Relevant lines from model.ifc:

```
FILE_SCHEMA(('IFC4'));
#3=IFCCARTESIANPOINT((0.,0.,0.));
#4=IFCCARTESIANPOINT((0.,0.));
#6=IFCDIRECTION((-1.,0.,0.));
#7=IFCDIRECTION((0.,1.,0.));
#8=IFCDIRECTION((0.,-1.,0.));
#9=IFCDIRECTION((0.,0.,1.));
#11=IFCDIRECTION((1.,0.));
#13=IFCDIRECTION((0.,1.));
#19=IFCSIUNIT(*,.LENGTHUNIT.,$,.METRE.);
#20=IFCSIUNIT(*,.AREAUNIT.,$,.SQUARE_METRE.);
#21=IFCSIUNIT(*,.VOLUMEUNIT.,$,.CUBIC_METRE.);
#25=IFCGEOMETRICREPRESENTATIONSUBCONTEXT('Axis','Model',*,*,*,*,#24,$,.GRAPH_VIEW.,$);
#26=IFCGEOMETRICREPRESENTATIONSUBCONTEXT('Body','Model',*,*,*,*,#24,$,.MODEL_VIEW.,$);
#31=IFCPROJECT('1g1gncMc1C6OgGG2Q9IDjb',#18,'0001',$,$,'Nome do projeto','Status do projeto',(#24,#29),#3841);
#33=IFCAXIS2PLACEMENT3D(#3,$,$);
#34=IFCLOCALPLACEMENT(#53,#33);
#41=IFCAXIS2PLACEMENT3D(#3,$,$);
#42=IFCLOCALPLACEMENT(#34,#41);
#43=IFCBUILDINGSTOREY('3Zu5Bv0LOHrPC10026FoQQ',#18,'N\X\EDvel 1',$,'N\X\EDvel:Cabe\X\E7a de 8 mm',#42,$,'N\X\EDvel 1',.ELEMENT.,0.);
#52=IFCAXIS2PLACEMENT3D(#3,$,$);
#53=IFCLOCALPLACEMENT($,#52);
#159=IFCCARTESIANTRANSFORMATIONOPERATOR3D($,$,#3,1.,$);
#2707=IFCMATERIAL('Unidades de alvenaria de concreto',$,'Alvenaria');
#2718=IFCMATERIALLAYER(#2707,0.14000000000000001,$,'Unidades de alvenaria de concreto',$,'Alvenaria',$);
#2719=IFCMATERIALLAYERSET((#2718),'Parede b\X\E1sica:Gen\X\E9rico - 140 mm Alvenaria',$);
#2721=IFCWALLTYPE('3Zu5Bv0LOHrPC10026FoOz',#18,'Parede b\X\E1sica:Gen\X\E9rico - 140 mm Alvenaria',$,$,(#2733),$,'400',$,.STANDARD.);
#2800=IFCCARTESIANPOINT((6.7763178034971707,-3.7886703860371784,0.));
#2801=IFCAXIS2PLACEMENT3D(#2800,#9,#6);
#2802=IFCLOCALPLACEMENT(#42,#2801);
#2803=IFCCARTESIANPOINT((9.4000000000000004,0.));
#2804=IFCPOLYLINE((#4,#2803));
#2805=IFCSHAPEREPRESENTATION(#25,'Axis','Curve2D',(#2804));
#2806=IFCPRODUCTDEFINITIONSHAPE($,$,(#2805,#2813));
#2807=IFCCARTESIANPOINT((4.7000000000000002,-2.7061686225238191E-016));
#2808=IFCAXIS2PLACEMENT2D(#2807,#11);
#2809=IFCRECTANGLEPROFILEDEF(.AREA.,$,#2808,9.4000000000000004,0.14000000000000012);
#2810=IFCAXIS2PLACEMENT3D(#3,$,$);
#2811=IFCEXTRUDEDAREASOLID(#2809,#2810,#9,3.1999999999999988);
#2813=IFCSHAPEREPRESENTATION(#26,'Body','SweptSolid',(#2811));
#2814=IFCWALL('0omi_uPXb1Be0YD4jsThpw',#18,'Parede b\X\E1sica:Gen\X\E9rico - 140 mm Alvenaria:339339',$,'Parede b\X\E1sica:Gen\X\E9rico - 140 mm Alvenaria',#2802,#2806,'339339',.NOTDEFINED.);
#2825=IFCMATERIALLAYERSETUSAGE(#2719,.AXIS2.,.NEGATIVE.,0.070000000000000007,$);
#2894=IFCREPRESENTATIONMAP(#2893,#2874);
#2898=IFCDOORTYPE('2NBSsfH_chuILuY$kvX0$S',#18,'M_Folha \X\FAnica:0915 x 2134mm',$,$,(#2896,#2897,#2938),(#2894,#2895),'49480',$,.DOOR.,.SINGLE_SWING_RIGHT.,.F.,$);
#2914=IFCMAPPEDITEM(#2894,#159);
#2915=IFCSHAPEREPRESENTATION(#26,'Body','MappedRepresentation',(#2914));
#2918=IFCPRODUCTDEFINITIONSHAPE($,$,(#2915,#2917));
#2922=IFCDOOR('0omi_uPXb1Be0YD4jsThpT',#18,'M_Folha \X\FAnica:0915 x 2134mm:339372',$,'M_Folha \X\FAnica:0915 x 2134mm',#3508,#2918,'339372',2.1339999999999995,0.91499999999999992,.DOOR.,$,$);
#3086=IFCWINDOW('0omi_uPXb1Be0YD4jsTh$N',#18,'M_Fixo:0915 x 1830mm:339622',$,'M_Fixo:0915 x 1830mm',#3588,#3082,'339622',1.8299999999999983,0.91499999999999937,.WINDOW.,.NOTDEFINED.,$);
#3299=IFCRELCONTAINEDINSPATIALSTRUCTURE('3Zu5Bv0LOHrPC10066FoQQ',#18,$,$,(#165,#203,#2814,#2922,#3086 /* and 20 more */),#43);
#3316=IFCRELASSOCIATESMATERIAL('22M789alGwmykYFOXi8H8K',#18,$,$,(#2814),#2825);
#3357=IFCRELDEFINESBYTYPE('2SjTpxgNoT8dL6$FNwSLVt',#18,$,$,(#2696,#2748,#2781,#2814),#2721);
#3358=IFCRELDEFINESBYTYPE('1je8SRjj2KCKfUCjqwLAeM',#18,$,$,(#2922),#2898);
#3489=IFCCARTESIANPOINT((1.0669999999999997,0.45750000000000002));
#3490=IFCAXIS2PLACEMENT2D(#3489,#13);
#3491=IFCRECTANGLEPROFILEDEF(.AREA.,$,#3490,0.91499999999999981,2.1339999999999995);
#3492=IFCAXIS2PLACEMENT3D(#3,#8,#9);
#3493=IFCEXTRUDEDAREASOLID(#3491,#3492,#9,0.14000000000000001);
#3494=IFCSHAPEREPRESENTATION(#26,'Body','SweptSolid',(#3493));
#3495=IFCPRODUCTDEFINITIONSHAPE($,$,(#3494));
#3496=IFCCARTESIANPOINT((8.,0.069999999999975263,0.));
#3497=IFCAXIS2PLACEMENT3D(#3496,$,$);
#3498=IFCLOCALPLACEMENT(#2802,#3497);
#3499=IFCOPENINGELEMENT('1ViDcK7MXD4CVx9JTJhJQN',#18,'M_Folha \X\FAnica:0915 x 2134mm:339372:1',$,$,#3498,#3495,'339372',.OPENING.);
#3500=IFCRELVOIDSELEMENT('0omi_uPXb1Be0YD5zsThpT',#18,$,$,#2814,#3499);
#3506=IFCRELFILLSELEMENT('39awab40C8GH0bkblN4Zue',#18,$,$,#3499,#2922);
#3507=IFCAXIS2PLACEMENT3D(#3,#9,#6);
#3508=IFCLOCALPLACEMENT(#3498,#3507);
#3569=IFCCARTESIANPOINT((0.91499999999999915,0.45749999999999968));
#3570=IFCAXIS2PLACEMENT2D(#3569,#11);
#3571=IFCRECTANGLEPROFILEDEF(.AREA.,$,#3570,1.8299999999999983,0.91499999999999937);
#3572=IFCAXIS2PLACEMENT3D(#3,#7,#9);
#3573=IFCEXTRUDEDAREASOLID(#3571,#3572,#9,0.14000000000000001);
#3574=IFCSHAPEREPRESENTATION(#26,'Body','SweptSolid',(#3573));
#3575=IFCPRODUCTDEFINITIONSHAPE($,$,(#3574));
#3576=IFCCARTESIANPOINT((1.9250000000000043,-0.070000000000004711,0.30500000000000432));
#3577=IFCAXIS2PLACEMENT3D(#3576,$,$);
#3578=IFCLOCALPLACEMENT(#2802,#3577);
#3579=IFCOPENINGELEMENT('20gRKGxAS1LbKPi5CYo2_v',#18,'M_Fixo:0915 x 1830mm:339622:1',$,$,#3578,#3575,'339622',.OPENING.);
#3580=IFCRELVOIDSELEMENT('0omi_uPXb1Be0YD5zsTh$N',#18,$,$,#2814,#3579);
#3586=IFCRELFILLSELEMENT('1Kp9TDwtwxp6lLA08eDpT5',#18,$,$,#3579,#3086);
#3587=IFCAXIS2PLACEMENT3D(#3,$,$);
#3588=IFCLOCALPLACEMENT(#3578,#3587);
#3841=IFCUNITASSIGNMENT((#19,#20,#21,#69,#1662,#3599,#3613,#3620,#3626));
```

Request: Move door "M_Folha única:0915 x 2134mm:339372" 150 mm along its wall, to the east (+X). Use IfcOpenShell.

```python
import ifcopenshell
import ifcopenshell.api.geometry
import ifcopenshell.util.placement
import ifcopenshell.util.unit

model = ifcopenshell.open("model.ifc")
unit_scale = ifcopenshell.util.unit.calculate_unit_scale(model)

door = model.by_id(2922)
opening = door.FillsVoids[0].RelatingOpeningElement
wall = opening.VoidsElements[0].RelatingBuildingElement

wall_matrix = ifcopenshell.util.placement.get_local_placement(wall.ObjectPlacement)
shift = wall_matrix[:3, 0] * -0.15 / unit_scale
before = ifcopenshell.util.placement.get_local_placement(door.ObjectPlacement)[:3, 3].copy()

# The door is placed relative to its opening, so it follows when the opening moves.
matrix = ifcopenshell.util.placement.get_local_placement(opening.ObjectPlacement)
matrix[:3, 3] += shift
ifcopenshell.api.geometry.edit_object_placement(
    model, product=opening, matrix=matrix, is_si=False, should_transform_children=True
)

after = ifcopenshell.util.placement.get_local_placement(door.ObjectPlacement)[:3, 3]
print("door moved by", (after - before).round(3) + 0.0)

model.write("model_rev.ifc")
```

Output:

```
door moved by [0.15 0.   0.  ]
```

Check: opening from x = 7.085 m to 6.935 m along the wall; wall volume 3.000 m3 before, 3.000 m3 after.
